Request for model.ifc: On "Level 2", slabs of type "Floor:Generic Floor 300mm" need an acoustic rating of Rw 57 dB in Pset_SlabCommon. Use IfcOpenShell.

First a look at what the model holds.

```python
import ifcopenshell
import ifcopenshell.util.element

model = ifcopenshell.open("model.ifc")
print(model.schema)
storey = next(s for s in model.by_type("IfcBuildingStorey") if s.Name == "Level 2")
slabs = [e for e in ifcopenshell.util.element.get_decomposition(storey) if e.is_a("IfcSlab")]
seen = {}
for e in slabs:
    element_type = ifcopenshell.util.element.get_type(e)
    key = (element_type.Name if element_type != e and element_type else None, ifcopenshell.util.element.get_pset(e, "Pset_SlabCommon", "AcousticRating"))
    seen[key] = seen.get(key, 0) + 1
for (name, value), count in sorted(seen.items(), key=str):
    print(count, "x", name, "|", value)
```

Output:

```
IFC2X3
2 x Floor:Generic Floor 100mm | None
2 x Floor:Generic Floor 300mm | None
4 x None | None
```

```python
import ifcopenshell
import ifcopenshell.api.pset
import ifcopenshell.util.element

model = ifcopenshell.open("model.ifc")

storey = next(s for s in model.by_type("IfcBuildingStorey") if s.Name == "Level 2")
slabs = [e for e in ifcopenshell.util.element.get_decomposition(storey) if e.is_a("IfcSlab")]

count = 0
for e in slabs:
    element_type = ifcopenshell.util.element.get_type(e)
    if element_type in (None, e) or element_type.Name != "Floor:Generic Floor 300mm":
        continue
    # add_pset returns the element's existing set when there is one.
    pset = ifcopenshell.api.pset.add_pset(model, product=e, name="Pset_SlabCommon")
    ifcopenshell.api.pset.edit_pset(model, pset=pset, properties={"AcousticRating": "Rw 57 dB"})
    count += 1

print(count, "slabs updated")

model.write("model_updated.ifc")
```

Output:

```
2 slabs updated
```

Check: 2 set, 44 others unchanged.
